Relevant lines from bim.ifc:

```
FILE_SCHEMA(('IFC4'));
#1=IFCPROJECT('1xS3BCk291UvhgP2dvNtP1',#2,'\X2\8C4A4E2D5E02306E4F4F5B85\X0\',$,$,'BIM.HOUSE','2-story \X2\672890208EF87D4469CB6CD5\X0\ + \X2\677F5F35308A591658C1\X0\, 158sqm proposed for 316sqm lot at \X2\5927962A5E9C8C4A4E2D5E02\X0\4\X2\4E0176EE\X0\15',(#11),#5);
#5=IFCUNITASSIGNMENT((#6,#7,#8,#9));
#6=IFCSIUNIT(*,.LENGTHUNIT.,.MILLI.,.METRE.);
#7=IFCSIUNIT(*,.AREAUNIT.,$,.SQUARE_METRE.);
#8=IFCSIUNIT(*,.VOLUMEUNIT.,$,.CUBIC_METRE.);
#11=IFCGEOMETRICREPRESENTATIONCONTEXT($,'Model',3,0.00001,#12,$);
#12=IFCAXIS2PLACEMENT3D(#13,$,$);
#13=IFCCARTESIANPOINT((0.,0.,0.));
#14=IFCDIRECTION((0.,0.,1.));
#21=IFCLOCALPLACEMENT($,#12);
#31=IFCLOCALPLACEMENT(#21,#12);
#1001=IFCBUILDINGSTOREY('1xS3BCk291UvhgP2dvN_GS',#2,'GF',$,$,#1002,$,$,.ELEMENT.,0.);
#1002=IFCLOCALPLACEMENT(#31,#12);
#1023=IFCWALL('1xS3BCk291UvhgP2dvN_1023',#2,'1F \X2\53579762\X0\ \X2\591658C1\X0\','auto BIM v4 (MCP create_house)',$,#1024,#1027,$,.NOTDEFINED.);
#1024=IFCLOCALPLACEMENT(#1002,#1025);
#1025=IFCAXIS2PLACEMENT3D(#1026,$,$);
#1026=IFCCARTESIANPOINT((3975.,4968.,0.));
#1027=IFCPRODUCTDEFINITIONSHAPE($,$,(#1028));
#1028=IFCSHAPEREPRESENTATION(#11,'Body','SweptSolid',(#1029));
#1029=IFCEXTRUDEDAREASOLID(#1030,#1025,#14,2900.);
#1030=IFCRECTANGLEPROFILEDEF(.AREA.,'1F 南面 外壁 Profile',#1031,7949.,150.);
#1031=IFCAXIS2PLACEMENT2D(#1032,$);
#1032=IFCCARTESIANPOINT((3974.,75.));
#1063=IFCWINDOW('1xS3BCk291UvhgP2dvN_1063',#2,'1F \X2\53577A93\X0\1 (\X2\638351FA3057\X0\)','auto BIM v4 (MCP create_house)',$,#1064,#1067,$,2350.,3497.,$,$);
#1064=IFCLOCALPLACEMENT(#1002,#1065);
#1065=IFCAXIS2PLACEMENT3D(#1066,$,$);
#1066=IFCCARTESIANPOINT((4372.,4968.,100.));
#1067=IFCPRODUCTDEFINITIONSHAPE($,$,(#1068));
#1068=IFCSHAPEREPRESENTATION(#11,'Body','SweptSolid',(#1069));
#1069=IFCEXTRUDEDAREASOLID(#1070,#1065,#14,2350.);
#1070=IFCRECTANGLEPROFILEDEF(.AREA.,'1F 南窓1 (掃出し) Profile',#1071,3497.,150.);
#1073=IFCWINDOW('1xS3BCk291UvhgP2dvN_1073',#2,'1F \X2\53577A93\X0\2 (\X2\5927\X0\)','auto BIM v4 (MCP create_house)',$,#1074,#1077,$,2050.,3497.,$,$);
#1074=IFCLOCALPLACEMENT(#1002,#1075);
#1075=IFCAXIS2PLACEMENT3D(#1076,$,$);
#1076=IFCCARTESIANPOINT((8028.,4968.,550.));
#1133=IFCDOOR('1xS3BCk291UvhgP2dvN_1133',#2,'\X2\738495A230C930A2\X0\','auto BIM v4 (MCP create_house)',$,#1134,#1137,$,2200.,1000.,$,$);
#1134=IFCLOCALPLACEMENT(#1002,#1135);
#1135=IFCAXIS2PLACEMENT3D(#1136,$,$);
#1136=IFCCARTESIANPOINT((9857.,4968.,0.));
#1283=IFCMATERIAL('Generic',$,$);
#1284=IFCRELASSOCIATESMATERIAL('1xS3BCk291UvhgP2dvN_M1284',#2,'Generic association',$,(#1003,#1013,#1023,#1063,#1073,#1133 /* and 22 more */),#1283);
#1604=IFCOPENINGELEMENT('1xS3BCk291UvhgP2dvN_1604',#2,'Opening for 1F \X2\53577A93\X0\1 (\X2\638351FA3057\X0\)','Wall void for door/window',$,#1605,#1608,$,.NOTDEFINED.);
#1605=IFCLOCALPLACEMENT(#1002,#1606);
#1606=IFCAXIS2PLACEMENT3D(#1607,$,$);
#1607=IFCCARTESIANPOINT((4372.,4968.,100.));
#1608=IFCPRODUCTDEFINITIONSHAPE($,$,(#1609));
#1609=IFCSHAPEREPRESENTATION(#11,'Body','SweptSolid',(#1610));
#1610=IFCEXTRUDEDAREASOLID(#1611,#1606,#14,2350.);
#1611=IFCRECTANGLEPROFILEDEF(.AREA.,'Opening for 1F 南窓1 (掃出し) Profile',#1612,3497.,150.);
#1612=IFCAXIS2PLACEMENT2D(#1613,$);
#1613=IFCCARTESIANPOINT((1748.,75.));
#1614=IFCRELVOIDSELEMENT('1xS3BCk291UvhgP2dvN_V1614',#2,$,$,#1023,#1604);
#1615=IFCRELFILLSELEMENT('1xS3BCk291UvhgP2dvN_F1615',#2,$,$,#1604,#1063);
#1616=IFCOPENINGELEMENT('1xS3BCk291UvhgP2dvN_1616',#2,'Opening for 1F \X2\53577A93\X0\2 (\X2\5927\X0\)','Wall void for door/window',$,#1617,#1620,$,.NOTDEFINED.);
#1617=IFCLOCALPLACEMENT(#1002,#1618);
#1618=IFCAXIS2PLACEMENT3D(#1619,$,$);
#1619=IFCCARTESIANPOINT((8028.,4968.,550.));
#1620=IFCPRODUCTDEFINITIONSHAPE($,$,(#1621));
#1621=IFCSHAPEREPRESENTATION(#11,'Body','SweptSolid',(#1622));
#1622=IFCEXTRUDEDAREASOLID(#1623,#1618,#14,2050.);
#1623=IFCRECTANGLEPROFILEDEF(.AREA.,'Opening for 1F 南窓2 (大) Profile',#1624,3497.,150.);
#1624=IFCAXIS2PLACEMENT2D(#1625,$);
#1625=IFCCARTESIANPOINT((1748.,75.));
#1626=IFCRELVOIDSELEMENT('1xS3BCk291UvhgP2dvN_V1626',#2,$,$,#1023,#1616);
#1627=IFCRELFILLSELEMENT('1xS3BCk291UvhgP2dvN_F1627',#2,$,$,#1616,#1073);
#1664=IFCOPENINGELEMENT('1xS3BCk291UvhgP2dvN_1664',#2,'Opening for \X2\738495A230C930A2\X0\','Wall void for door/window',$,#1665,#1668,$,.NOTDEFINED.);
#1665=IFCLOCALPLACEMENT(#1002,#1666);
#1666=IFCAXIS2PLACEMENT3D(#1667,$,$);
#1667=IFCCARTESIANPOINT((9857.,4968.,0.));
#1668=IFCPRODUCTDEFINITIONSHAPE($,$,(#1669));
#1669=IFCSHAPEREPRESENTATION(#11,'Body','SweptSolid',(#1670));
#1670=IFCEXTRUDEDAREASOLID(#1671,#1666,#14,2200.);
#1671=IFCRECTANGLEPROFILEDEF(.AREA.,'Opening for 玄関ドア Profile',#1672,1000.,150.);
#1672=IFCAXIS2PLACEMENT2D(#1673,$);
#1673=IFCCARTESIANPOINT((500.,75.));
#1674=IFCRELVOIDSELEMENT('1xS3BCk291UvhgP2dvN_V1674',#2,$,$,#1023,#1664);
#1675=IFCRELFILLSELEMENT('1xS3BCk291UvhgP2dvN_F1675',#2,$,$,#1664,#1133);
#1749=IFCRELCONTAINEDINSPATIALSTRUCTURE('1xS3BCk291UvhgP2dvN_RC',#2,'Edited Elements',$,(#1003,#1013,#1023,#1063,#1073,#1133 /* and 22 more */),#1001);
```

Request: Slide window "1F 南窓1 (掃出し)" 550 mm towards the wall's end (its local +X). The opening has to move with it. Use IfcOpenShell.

```python
import ifcopenshell
import ifcopenshell.api.geometry
import ifcopenshell.util.placement

model = ifcopenshell.open("bim.ifc")

window = model.by_id(1063)
opening = window.FillsVoids[0].RelatingOpeningElement
wall = opening.VoidsElements[0].RelatingBuildingElement

wall_matrix = ifcopenshell.util.placement.get_local_placement(wall.ObjectPlacement)
shift = wall_matrix[:3, 0] * 550.0
before = ifcopenshell.util.placement.get_local_placement(window.ObjectPlacement)[:3, 3].copy()

# The window is not placed relative to its opening, so move both.
for product in (opening, window):
    matrix = ifcopenshell.util.placement.get_local_placement(product.ObjectPlacement)
    matrix[:3, 3] += shift
    ifcopenshell.api.geometry.edit_object_placement(model, product=product, matrix=matrix, is_si=False)

after = ifcopenshell.util.placement.get_local_placement(window.ObjectPlacement)[:3, 3]
print("window moved by", (after - before).round(3) + 0.0)

model.write("bim_v2.ifc")
```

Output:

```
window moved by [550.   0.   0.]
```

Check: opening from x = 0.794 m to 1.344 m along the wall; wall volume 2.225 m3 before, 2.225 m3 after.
